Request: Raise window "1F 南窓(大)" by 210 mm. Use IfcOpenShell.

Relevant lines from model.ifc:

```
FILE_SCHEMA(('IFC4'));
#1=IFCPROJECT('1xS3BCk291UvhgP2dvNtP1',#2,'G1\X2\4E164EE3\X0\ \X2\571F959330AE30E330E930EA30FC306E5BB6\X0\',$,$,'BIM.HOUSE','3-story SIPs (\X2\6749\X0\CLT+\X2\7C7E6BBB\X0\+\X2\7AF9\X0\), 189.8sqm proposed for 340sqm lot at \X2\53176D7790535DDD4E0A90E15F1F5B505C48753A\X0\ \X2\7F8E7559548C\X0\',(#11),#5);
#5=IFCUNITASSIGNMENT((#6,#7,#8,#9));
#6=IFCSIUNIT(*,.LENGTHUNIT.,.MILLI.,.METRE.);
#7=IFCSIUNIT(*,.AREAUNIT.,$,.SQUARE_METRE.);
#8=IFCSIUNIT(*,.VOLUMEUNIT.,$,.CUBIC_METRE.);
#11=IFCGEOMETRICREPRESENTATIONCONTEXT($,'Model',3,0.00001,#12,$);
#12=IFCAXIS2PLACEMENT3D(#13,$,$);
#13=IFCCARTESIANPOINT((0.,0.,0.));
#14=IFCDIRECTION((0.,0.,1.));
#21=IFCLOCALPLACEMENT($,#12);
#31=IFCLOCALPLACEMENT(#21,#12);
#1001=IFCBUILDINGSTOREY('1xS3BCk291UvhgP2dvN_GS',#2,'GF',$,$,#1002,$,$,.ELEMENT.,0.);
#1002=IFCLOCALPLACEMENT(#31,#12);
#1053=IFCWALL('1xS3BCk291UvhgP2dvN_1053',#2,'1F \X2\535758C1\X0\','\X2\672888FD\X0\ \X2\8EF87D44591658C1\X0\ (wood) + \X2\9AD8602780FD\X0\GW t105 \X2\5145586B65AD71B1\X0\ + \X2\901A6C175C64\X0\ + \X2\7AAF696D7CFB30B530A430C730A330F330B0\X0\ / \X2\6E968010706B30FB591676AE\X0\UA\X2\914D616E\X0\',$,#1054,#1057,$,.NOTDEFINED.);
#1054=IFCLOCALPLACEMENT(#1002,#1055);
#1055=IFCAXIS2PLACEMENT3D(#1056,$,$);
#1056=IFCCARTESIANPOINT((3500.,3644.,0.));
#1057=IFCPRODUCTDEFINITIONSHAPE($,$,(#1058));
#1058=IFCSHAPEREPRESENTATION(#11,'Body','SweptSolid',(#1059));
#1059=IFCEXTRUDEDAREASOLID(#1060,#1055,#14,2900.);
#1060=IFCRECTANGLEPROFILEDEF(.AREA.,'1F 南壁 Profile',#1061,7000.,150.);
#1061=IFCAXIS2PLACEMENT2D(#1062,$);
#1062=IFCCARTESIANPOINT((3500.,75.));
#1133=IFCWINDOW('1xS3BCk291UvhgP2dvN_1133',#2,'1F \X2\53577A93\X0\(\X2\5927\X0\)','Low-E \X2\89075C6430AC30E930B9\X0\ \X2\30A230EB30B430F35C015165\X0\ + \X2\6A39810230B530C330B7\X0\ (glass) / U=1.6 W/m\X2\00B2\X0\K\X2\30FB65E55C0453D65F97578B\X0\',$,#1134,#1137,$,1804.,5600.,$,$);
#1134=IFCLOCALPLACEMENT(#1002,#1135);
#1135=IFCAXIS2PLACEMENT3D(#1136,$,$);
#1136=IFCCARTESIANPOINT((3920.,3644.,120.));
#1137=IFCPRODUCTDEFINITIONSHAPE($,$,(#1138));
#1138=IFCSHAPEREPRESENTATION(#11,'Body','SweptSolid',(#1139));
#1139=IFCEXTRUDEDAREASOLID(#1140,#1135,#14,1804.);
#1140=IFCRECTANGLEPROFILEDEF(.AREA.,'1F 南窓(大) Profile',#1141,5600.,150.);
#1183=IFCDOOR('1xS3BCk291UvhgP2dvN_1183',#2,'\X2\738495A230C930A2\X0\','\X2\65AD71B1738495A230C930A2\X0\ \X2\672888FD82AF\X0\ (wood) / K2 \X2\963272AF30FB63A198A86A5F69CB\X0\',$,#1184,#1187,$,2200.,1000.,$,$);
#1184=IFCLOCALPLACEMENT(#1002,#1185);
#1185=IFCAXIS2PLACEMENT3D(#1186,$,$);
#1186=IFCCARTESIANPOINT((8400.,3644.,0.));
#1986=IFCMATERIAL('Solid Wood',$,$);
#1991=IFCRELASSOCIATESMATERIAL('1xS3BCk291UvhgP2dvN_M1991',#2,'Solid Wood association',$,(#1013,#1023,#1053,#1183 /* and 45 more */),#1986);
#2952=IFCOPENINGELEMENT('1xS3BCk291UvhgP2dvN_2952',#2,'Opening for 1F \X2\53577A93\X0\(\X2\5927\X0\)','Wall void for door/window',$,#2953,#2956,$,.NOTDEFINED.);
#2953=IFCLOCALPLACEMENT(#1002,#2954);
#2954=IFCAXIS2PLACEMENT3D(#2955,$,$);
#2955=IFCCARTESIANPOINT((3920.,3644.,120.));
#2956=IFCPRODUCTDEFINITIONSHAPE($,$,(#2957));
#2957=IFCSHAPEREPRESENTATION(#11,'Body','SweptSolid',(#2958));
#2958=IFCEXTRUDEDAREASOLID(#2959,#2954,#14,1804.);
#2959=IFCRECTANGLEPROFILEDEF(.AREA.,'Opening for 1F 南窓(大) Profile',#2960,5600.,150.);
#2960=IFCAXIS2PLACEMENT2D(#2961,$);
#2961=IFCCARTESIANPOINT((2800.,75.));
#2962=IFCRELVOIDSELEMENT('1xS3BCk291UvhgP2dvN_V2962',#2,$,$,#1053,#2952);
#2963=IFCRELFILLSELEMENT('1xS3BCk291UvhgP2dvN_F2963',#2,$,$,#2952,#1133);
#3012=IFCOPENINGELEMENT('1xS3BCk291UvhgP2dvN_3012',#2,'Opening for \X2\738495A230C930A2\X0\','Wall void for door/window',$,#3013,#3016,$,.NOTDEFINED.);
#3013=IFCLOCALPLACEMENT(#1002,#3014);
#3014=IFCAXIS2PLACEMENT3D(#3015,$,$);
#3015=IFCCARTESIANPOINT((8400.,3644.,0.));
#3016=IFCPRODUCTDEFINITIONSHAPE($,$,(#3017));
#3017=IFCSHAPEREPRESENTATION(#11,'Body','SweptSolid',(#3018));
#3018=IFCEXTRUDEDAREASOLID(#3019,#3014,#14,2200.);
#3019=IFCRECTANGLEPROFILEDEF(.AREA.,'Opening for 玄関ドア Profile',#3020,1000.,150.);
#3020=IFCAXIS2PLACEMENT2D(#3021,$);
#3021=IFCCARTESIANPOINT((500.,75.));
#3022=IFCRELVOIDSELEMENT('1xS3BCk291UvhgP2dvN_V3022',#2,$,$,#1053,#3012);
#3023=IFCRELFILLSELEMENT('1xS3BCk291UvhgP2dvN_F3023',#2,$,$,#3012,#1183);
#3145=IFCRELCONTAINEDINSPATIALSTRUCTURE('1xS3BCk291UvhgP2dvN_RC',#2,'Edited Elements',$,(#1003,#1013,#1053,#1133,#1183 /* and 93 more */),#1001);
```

```python
import numpy as np
import ifcopenshell
import ifcopenshell.api.geometry
import ifcopenshell.util.placement
import ifcopenshell.util.unit

model = ifcopenshell.open("model.ifc")
unit_scale = ifcopenshell.util.unit.calculate_unit_scale(model)

window = model.by_id(1133)
opening = window.FillsVoids[0].RelatingOpeningElement
dz = 210.0

shift = np.array([0.0, 0.0, dz])
# The window is not placed relative to its opening, so move both.
for product in (opening, window):
    matrix = ifcopenshell.util.placement.get_local_placement(product.ObjectPlacement)
    matrix[:3, 3] += shift
    ifcopenshell.api.geometry.edit_object_placement(model, product=product, matrix=matrix, is_si=False)

print(f"moved by {dz * unit_scale:+.3f} m")

model.write("model-out.ifc")
```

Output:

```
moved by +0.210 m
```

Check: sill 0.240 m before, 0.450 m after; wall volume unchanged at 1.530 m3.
